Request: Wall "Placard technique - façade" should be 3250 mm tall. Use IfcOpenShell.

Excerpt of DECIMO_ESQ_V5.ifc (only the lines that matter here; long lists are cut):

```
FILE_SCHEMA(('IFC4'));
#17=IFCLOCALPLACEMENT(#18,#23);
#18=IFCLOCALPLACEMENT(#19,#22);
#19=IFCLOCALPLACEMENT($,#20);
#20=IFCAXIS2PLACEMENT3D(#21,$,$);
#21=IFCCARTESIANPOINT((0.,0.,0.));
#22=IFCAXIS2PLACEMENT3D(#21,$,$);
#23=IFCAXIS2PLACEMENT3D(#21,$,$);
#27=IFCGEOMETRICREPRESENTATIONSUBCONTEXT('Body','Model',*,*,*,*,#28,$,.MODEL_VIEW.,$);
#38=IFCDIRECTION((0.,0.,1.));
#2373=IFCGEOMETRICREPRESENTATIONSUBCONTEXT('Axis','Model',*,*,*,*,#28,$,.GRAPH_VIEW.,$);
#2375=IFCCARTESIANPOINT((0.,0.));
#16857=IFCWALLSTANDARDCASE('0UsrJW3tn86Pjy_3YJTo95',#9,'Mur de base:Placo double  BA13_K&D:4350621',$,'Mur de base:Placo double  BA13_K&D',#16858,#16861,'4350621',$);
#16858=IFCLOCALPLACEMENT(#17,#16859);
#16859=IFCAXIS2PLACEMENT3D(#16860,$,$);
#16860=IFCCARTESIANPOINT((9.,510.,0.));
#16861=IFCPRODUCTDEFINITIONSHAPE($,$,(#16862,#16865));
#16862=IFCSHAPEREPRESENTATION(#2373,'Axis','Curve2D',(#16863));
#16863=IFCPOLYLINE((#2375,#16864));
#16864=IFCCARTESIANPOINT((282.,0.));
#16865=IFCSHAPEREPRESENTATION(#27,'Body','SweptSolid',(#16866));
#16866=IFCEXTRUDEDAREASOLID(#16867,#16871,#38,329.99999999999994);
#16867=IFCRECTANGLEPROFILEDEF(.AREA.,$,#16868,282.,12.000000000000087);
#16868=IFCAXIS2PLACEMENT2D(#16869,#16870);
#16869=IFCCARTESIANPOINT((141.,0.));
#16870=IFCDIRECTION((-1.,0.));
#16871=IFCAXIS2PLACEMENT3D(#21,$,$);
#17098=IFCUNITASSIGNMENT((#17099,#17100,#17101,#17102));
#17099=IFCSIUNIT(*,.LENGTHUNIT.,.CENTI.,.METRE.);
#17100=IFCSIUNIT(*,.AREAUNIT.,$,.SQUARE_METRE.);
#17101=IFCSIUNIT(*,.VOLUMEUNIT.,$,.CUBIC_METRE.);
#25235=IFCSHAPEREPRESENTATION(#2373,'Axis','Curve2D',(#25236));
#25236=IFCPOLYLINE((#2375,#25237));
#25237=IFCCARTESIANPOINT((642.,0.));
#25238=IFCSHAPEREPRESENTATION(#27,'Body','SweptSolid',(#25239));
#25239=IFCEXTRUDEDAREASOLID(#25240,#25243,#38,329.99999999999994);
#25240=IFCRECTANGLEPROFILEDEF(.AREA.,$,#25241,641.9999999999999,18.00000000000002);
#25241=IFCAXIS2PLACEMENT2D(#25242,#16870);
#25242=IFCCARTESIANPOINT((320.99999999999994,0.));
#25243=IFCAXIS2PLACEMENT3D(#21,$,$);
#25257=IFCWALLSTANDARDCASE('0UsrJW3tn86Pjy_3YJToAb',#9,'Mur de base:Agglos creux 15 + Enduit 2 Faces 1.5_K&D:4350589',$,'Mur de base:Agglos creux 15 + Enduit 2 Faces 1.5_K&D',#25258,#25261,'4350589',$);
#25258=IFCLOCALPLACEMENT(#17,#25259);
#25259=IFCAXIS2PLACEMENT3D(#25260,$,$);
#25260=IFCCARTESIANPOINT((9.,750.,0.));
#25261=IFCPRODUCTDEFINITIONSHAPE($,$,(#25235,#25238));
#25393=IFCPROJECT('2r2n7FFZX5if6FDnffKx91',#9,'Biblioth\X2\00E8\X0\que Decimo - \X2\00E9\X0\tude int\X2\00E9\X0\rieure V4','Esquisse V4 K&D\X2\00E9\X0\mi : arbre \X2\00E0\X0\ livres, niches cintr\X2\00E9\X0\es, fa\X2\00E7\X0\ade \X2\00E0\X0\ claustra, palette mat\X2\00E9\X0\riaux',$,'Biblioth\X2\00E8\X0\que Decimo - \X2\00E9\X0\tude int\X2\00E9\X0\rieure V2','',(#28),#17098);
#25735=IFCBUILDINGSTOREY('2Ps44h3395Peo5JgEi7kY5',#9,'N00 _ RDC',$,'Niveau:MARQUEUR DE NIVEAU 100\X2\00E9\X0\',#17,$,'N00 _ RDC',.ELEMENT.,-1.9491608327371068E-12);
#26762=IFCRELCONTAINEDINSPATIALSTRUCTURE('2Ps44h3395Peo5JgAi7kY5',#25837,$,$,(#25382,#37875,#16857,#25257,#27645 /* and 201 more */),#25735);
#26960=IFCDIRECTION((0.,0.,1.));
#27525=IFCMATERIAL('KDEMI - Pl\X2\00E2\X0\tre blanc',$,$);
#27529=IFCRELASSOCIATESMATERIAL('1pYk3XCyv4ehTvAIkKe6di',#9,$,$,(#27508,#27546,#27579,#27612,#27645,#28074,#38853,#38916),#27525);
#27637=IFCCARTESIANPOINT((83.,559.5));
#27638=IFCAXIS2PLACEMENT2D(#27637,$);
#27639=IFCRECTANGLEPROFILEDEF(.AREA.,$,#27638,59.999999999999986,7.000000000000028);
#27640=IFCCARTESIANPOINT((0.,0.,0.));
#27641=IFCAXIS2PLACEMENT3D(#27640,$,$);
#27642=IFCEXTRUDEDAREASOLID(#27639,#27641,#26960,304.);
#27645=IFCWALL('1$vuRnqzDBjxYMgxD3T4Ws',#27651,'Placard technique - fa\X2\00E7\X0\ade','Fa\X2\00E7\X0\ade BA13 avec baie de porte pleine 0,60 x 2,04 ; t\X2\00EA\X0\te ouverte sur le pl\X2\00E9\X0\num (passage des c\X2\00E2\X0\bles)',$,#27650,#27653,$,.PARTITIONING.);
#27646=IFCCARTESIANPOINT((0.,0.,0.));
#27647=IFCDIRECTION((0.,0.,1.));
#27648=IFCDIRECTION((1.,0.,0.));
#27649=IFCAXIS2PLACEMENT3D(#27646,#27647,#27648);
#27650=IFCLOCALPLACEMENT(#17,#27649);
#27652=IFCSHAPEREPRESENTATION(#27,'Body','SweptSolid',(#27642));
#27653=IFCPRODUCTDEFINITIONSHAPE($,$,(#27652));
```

```python
import ifcopenshell
import ifcopenshell.geom
import ifcopenshell.util.representation
import ifcopenshell.util.shape
import ifcopenshell.util.unit

model = ifcopenshell.open("DECIMO_ESQ_V5.ifc")
unit_scale = ifcopenshell.util.unit.calculate_unit_scale(model)
settings = ifcopenshell.geom.settings()


def volume(element):
    """Net volume in cubic metres, openings subtracted."""
    shape = ifcopenshell.geom.create_shape(settings, element)
    return ifcopenshell.util.shape.get_volume(shape.geometry)


wall = model.by_guid("1$vuRnqzDBjxYMgxD3T4Ws")
before = volume(wall)

body = ifcopenshell.util.representation.get_representation(wall, "Model", "Body")
solid = body.Items[0]
old_height = solid.Depth
solid.Depth = 3.25 / unit_scale
after = volume(wall)

print(f"height {old_height:g} -> {solid.Depth:g}, volume {before:.3f} -> {after:.3f} m3")

model.write("DECIMO_ESQ_V5_rev.ifc")
```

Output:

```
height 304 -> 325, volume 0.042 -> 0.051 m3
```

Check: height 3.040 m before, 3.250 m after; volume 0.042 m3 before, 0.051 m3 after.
